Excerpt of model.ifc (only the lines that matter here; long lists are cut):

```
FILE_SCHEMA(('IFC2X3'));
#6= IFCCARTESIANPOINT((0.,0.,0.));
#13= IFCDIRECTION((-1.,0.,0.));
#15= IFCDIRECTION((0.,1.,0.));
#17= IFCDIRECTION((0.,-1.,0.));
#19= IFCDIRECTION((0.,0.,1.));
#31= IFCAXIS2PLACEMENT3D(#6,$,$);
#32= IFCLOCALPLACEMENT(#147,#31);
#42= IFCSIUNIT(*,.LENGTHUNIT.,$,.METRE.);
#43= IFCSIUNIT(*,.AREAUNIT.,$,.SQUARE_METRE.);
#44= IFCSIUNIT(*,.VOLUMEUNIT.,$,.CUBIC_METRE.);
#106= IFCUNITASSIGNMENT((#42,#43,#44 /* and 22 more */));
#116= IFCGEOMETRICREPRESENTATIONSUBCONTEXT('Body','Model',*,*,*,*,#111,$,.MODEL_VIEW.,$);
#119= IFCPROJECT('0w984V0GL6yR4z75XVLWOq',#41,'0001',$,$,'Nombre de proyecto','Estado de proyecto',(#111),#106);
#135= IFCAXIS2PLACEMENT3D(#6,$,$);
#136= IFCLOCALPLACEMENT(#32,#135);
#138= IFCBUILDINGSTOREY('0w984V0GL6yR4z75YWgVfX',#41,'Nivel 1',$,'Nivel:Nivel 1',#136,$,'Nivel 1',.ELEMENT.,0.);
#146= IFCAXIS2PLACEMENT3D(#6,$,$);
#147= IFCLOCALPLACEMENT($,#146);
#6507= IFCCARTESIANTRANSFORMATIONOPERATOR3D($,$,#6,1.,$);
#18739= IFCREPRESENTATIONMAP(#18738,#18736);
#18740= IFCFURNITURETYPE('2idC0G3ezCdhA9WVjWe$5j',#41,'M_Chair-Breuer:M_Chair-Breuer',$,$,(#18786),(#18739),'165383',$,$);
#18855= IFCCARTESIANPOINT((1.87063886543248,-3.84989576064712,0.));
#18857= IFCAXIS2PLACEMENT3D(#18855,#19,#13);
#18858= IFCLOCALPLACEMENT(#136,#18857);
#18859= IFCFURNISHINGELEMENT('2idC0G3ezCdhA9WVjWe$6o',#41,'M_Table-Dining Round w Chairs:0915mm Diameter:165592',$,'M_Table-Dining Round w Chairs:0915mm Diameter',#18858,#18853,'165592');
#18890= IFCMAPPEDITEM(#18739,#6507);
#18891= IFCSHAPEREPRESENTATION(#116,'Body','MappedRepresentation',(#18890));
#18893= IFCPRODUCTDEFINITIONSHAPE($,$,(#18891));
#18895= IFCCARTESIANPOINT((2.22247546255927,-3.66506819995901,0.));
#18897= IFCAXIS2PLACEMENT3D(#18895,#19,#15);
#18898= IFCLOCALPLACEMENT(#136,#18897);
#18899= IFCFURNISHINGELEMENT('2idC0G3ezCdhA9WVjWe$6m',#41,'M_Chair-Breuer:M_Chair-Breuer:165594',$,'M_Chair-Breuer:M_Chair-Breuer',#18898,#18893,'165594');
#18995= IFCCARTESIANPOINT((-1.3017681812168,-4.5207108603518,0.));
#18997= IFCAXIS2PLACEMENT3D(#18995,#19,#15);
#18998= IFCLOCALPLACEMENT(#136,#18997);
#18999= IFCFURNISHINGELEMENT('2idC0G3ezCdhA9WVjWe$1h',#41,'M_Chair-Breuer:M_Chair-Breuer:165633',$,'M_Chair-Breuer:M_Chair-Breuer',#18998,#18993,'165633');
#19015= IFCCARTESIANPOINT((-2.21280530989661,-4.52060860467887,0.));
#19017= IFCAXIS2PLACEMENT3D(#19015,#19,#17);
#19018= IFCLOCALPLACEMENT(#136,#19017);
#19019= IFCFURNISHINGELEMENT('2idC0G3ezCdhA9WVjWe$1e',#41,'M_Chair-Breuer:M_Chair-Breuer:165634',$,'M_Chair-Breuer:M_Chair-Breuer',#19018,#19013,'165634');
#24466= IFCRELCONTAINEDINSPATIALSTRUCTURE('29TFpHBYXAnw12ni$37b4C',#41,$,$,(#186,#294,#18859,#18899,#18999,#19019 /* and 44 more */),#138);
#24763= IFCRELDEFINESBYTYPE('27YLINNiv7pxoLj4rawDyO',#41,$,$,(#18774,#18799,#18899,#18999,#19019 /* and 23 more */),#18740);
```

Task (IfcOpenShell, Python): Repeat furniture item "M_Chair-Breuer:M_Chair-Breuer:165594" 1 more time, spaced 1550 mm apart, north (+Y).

```python
import numpy as np
import ifcopenshell
import ifcopenshell.api.geometry
import ifcopenshell.api.root
import ifcopenshell.util.element
import ifcopenshell.util.placement
import ifcopenshell.util.unit

model = ifcopenshell.open("model.ifc")
unit_scale = ifcopenshell.util.unit.calculate_unit_scale(model)


def reuse_history(source, copy):
    """copy_class also copies each property set's owner history, people and application; keep the originals."""
    for rel in copy.IsDefinedBy:
        if rel.is_a("IfcRelDefinesByProperties") and (history := rel.RelatingPropertyDefinition.OwnerHistory):
            rel.RelatingPropertyDefinition.OwnerHistory = source.OwnerHistory
            ifcopenshell.util.element.remove_deep2(model, history)


source = model.by_id(18899)
base = ifcopenshell.util.placement.get_local_placement(source.ObjectPlacement)
step = np.array([0.0, 1.0, 0.0]) * 1.55 / unit_scale

for i in range(1, 2):
    copy = ifcopenshell.api.root.copy_class(model, product=source)
    copy.Representation = ifcopenshell.util.element.copy_deep(
        model, source.Representation, exclude=["IfcGeometricRepresentationContext", "IfcRepresentationMap"]
    )
    copy.Name = "M_Chair-Breuer:M_Chair-Breuer"
    copy.Tag = None
    reuse_history(source, copy)
    matrix = base.copy()
    matrix[:3, 3] += i * step
    print("added at", matrix[:3, 3].round(3) + 0.0)
    ifcopenshell.api.geometry.edit_object_placement(model, product=copy, matrix=matrix, is_si=False)

model.write("model-out.ifc")
```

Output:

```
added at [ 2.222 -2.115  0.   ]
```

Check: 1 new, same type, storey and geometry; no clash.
